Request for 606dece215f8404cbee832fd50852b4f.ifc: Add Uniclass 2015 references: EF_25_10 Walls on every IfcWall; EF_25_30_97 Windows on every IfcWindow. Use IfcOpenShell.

First a look at what the model holds.

```python
import ifcopenshell

model = ifcopenshell.open("606dece215f8404cbee832fd50852b4f.ifc")
print(model.schema)
print("classifications:", [c.Name for c in model.by_type("IfcClassification")])
for ifc_class in ("IfcDoor", "IfcRoof", "IfcStair", "IfcWall", "IfcWindow"):
    print(ifc_class, len(model.by_type(ifc_class)))
```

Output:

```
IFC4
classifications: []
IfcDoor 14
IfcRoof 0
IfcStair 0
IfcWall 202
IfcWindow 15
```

```python
import ifcopenshell
import ifcopenshell.api.classification

model = ifcopenshell.open("606dece215f8404cbee832fd50852b4f.ifc")

system = ifcopenshell.api.classification.add_classification(model, classification="Uniclass 2015")

codes = {
    "IfcWall": ("EF_25_10", "Walls"),
    "IfcWindow": ("EF_25_30_97", "Windows"),
}
for ifc_class, (code, name) in codes.items():
    products = model.by_type(ifc_class)
    ifcopenshell.api.classification.add_reference(
        model, products=products, classification=system, identification=code, name=name
    )
    print(code, len(products))

model.write("606dece215f8404cbee832fd50852b4f_v2.ifc")
```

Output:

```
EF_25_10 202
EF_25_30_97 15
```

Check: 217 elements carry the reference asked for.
